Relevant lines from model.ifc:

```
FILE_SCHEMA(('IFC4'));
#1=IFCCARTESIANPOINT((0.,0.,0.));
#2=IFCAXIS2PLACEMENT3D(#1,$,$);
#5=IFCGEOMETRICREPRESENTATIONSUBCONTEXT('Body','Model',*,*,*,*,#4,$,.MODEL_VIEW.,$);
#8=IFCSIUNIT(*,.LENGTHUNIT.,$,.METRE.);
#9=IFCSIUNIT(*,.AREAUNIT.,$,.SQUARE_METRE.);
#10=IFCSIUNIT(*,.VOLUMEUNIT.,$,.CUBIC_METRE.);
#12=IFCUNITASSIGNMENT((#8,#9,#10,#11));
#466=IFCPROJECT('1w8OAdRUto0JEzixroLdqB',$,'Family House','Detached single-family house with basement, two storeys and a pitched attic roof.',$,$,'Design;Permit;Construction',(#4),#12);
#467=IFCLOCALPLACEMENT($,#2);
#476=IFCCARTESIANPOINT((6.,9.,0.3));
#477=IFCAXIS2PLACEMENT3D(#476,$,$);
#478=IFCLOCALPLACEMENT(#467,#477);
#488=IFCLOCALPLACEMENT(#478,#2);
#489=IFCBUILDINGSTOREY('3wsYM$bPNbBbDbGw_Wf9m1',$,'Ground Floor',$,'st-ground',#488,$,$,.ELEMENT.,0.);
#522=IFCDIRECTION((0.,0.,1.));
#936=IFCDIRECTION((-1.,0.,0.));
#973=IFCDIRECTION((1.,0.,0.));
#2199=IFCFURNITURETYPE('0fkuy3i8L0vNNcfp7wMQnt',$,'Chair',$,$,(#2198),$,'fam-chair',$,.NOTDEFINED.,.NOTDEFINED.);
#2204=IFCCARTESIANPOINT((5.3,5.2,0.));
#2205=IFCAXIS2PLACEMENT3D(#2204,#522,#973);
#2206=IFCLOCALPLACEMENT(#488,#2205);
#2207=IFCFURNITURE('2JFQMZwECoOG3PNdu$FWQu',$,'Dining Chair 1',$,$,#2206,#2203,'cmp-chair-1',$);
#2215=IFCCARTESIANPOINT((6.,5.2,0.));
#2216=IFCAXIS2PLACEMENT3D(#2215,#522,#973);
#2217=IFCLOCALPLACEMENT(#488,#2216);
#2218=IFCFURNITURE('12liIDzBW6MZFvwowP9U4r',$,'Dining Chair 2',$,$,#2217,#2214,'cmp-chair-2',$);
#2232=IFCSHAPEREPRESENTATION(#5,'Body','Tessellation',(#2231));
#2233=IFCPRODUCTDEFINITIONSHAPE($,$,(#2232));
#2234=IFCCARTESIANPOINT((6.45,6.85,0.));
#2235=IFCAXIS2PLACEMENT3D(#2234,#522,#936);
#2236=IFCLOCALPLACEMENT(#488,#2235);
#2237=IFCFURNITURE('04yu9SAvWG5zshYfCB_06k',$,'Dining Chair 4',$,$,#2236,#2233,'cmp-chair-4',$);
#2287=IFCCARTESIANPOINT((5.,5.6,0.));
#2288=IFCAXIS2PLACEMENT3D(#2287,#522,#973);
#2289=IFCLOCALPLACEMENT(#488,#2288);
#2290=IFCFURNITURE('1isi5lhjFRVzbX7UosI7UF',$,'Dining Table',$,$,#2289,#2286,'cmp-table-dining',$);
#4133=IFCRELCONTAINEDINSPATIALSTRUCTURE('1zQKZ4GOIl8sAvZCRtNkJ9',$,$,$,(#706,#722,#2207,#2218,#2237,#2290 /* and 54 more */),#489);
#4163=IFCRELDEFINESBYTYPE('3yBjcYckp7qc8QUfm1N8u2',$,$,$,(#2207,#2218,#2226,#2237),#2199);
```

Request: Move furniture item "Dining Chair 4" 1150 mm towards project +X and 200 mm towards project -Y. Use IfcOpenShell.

```python
import ifcopenshell
import ifcopenshell.api.geometry
import ifcopenshell.util.placement

model = ifcopenshell.open("model.ifc")

item = model.by_guid("04yu9SAvWG5zshYfCB_06k")
matrix = ifcopenshell.util.placement.get_local_placement(item.ObjectPlacement)
matrix[0, 3] += 1.15
matrix[1, 3] -= 0.2
ifcopenshell.api.geometry.edit_object_placement(model, product=item, matrix=matrix, is_si=False)

print(ifcopenshell.util.placement.get_local_placement(item.ObjectPlacement).round(3) + 0.0)

model.write("model_v2.ifc")
```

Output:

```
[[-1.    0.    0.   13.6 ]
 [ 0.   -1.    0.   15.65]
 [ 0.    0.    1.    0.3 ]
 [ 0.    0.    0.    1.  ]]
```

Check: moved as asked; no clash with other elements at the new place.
